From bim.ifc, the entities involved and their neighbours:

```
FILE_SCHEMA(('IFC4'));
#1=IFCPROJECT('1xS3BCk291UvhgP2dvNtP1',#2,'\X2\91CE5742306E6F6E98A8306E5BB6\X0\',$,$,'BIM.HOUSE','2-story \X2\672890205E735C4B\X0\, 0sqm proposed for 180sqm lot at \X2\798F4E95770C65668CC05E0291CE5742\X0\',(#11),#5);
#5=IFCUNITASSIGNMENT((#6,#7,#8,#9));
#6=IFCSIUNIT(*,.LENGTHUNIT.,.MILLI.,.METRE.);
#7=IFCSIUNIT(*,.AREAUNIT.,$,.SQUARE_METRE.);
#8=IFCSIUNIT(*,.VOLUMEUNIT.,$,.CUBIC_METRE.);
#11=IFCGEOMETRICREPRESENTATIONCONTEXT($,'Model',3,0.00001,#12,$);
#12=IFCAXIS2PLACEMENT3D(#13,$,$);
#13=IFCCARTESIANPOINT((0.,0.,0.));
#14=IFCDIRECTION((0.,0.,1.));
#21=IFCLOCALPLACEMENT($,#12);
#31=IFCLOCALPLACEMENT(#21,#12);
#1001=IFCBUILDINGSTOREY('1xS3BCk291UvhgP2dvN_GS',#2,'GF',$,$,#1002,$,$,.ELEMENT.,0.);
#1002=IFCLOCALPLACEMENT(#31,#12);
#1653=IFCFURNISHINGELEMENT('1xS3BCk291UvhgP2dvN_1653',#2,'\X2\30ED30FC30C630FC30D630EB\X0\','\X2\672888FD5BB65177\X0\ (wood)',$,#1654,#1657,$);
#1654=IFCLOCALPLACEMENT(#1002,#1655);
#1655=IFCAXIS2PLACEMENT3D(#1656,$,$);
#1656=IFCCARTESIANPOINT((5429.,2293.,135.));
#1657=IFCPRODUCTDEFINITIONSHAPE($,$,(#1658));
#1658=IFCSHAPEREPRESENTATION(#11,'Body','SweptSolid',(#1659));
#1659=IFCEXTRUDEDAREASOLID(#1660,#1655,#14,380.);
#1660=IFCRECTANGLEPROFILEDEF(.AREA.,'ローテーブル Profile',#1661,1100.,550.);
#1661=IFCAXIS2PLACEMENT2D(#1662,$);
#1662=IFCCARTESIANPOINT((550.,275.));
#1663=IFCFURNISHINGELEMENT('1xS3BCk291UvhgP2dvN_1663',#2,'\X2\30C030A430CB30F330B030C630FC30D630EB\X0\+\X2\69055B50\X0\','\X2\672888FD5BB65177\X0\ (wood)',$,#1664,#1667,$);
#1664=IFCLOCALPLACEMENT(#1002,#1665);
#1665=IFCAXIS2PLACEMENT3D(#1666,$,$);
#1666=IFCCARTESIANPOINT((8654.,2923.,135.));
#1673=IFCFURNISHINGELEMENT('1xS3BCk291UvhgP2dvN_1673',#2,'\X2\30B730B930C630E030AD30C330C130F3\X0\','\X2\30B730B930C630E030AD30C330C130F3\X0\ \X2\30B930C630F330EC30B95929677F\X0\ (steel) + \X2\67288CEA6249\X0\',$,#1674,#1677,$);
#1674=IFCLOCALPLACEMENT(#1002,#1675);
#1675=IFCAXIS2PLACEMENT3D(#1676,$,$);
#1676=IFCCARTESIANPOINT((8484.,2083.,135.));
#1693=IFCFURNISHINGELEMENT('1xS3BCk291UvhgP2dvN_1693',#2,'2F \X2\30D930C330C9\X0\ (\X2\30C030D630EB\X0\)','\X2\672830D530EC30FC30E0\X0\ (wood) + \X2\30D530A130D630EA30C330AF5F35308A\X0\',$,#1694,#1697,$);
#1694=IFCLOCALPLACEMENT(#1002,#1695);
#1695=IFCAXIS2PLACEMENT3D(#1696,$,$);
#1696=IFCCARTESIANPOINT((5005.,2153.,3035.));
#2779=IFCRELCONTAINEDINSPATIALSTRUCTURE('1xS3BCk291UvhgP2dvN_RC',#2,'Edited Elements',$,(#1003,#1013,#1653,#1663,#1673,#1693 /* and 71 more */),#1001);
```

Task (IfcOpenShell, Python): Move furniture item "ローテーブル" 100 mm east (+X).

```python
import ifcopenshell
import ifcopenshell.api.geometry
import ifcopenshell.util.placement
import ifcopenshell.util.unit

model = ifcopenshell.open("bim.ifc")
unit_scale = ifcopenshell.util.unit.calculate_unit_scale(model)

item = model.by_guid("1xS3BCk291UvhgP2dvN_1653")
matrix = ifcopenshell.util.placement.get_local_placement(item.ObjectPlacement)
matrix[0, 3] += 0.1 / unit_scale
ifcopenshell.api.geometry.edit_object_placement(model, product=item, matrix=matrix, is_si=False)

print(ifcopenshell.util.placement.get_local_placement(item.ObjectPlacement).round(3) + 0.0)

model.write("bim_v2.ifc")
```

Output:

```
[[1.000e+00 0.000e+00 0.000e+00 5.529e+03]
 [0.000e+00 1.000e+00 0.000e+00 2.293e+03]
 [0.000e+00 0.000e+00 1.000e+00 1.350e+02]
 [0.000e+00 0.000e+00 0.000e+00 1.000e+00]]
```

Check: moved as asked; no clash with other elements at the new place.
